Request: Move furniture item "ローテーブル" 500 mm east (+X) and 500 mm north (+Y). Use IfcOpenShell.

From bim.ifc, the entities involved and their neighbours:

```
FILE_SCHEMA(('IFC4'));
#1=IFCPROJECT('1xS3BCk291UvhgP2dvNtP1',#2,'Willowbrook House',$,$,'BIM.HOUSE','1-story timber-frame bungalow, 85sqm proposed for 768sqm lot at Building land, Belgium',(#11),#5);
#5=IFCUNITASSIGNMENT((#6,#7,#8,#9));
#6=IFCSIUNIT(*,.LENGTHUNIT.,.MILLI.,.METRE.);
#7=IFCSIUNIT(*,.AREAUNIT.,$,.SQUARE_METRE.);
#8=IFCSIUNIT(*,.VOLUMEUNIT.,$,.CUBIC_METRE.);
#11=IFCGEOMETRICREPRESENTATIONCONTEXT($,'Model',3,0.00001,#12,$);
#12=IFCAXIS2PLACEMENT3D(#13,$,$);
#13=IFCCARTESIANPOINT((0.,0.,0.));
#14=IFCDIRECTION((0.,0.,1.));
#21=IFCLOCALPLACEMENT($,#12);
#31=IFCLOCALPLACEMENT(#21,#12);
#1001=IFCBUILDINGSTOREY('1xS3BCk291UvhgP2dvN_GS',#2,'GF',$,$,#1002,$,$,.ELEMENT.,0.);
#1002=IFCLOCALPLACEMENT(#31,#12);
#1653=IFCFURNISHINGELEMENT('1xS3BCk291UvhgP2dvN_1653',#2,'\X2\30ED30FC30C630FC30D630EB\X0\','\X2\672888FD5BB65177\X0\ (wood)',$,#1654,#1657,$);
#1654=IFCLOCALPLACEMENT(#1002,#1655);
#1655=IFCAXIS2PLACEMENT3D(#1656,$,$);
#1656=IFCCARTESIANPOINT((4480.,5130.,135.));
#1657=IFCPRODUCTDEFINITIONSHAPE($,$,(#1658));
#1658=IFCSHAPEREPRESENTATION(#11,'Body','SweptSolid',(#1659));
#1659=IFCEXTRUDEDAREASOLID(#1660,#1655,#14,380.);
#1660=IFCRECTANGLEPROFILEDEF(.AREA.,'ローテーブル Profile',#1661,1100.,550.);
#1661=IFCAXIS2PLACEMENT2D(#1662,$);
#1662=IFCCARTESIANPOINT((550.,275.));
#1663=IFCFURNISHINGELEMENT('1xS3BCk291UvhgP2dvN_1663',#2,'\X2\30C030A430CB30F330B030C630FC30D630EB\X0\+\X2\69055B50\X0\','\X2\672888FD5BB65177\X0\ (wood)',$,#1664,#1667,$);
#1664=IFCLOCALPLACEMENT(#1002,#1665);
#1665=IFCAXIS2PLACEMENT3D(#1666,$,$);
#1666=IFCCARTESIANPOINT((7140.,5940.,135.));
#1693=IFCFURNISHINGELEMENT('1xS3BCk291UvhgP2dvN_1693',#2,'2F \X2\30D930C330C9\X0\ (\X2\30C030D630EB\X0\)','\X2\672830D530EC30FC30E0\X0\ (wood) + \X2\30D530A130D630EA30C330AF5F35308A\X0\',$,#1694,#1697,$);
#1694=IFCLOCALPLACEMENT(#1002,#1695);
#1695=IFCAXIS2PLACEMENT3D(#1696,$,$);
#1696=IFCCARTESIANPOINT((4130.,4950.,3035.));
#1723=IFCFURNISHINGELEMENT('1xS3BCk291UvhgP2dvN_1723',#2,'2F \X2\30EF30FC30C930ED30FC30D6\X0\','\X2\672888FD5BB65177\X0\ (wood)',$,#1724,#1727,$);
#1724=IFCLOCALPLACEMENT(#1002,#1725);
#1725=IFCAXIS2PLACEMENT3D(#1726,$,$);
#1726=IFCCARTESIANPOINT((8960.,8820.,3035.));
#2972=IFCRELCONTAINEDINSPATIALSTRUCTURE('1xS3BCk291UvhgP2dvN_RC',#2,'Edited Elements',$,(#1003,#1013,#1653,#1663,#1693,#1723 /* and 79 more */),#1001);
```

```python
import ifcopenshell
import ifcopenshell.api.geometry
import ifcopenshell.util.placement

model = ifcopenshell.open("bim.ifc")

item = model.by_guid("1xS3BCk291UvhgP2dvN_1653")
matrix = ifcopenshell.util.placement.get_local_placement(item.ObjectPlacement)
matrix[0, 3] += 500.0
matrix[1, 3] += 500.0
ifcopenshell.api.geometry.edit_object_placement(model, product=item, matrix=matrix, is_si=False)

print(ifcopenshell.util.placement.get_local_placement(item.ObjectPlacement).round(3) + 0.0)

model.write("bim_updated.ifc")
```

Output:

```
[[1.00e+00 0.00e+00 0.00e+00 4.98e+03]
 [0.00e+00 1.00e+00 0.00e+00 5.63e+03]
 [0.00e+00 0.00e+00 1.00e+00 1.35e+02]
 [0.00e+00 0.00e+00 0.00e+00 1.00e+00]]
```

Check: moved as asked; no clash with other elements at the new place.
